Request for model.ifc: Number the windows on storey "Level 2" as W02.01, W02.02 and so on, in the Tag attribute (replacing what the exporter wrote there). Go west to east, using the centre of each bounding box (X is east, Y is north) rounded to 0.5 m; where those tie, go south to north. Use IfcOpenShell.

First a look at what the model holds.

```python
import ifcopenshell
import ifcopenshell.util.element
import ifcopenshell.util.placement

model = ifcopenshell.open("model.ifc")
print(model.schema)
storey = next(s for s in model.by_type("IfcBuildingStorey") if s.Name == "Level 2")
windows = [e for e in ifcopenshell.util.element.get_decomposition(storey) if e.is_a("IfcWindow")]
for e in sorted(windows, key=lambda e: e.id()):
    origin = ifcopenshell.util.placement.get_local_placement(e.ObjectPlacement)[:3, 3]
    print(e.id(), e.Tag, e.Name, origin.round(2) + 0.0, sep=" | ")
```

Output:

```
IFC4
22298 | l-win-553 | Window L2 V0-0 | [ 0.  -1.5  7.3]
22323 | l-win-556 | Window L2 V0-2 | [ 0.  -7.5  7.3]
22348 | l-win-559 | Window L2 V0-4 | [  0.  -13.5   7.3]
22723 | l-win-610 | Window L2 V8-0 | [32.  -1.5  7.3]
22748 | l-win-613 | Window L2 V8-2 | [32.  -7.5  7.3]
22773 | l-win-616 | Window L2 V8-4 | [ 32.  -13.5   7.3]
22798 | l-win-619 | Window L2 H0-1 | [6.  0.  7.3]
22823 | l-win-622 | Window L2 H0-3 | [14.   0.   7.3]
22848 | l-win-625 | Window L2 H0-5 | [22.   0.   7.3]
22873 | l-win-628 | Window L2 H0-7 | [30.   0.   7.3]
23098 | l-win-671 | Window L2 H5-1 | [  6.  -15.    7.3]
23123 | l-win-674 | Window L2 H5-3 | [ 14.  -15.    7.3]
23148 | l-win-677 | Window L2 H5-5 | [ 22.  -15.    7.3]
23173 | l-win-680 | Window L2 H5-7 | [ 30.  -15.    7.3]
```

```python
import ifcopenshell
import ifcopenshell.geom
import ifcopenshell.util.element
import ifcopenshell.util.shape

model = ifcopenshell.open("model.ifc")
settings = ifcopenshell.geom.settings()
settings.set("use-world-coords", True)


def centre(element):
    shape = ifcopenshell.geom.create_shape(settings, element)
    return ifcopenshell.util.shape.get_bbox_centroid(shape.geometry)


storey = next(s for s in model.by_type("IfcBuildingStorey") if s.Name == "Level 2")
windows = [e for e in ifcopenshell.util.element.get_decomposition(storey) if e.is_a("IfcWindow")]

# Insertion points can sit at a corner or the storey origin, so sort by the geometry (in metres).
centres = {e: centre(e) for e in windows}
windows.sort(key=lambda e: (round(centres[e][0] / 0.5), centres[e][1]))

for i, e in enumerate(windows, start=1):
    number = f"W02.{i:02d}"
    e.Tag = number
    print(e.id(), number)

model.write("model-out.ifc")
```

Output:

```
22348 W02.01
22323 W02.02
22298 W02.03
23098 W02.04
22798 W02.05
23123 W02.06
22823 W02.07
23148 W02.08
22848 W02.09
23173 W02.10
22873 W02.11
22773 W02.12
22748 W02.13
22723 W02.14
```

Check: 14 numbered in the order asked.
